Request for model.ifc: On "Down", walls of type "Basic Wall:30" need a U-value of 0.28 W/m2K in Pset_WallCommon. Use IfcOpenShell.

First a look at what the model holds.

```python
import ifcopenshell
import ifcopenshell.util.element

model = ifcopenshell.open("model.ifc")
print(model.schema)
storey = next(s for s in model.by_type("IfcBuildingStorey") if s.Name == "Down")
walls = [e for e in ifcopenshell.util.element.get_decomposition(storey) if e.is_a("IfcWall")]
seen = {}
for e in walls:
    element_type = ifcopenshell.util.element.get_type(e)
    key = (element_type.Name if element_type != e and element_type else None, ifcopenshell.util.element.get_pset(e, "Pset_WallCommon", "ThermalTransmittance"))
    seen[key] = seen.get(key, 0) + 1
for (name, value), count in sorted(seen.items(), key=str):
    print(count, "x", name, "|", value)
```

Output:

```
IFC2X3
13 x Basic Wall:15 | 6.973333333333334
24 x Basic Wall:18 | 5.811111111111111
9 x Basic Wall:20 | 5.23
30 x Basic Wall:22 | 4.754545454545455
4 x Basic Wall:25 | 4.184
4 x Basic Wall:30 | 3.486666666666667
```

```python
import ifcopenshell
import ifcopenshell.api.pset
import ifcopenshell.util.element

model = ifcopenshell.open("model.ifc")

storey = next(s for s in model.by_type("IfcBuildingStorey") if s.Name == "Down")
walls = [e for e in ifcopenshell.util.element.get_decomposition(storey) if e.is_a("IfcWall")]

count = 0
for e in walls:
    element_type = ifcopenshell.util.element.get_type(e)
    if element_type in (None, e) or element_type.Name != "Basic Wall:30":
        continue
    # add_pset returns the element's existing set when there is one.
    pset = ifcopenshell.api.pset.add_pset(model, product=e, name="Pset_WallCommon")
    ifcopenshell.api.pset.edit_pset(model, pset=pset, properties={"ThermalTransmittance": 0.28})
    count += 1

print(count, "walls updated")

model.write("model_updated.ifc")
```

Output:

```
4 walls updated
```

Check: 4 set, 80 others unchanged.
